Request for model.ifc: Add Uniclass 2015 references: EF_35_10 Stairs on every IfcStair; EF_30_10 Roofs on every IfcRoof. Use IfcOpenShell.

First a look at what the model holds.

```python
import ifcopenshell

model = ifcopenshell.open("model.ifc")
print(model.schema)
print("classifications:", [c.Name for c in model.by_type("IfcClassification")])
for ifc_class in ("IfcDoor", "IfcRoof", "IfcStair", "IfcWall", "IfcWindow"):
    print(ifc_class, len(model.by_type(ifc_class)))
```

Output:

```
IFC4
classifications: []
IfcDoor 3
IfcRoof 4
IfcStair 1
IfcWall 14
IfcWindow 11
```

```python
import ifcopenshell
import ifcopenshell.api.classification

model = ifcopenshell.open("model.ifc")

system = ifcopenshell.api.classification.add_classification(model, classification="Uniclass 2015")

codes = {
    "IfcStair": ("EF_35_10", "Stairs"),
    "IfcRoof": ("EF_30_10", "Roofs"),
}
for ifc_class, (code, name) in codes.items():
    products = model.by_type(ifc_class)
    ifcopenshell.api.classification.add_reference(
        model, products=products, classification=system, identification=code, name=name
    )
    print(code, len(products))

model.write("model_v2.ifc")
```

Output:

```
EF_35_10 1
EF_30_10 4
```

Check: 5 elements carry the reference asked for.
